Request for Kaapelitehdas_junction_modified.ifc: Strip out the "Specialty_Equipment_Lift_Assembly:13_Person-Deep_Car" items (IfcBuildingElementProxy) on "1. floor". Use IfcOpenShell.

First a look at what the model holds.

```python
import ifcopenshell
import ifcopenshell.util.element

model = ifcopenshell.open("Kaapelitehdas_junction_modified.ifc")
print(model.schema)
storey = next(s for s in model.by_type("IfcBuildingStorey") if s.Name == "1. floor")
proxies = [e for e in ifcopenshell.util.element.get_decomposition(storey) if e.is_a("IfcBuildingElementProxy")]
seen = {}
for e in proxies:
    element_type = ifcopenshell.util.element.get_type(e)
    name = element_type.Name if element_type not in (None, e) else None
    seen[name] = seen.get(name, 0) + 1
for name, count in sorted(seen.items(), key=str):
    print(count, "x", name)
```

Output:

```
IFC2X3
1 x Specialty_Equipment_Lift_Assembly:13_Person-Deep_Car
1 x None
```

```python
import ifcopenshell
import ifcopenshell.api.root
import ifcopenshell.util.element

model = ifcopenshell.open("Kaapelitehdas_junction_modified.ifc")

storey = next(s for s in model.by_type("IfcBuildingStorey") if s.Name == "1. floor")
proxies = [e for e in ifcopenshell.util.element.get_decomposition(storey) if e.is_a("IfcBuildingElementProxy")]
targets = [e for e in proxies if (t := ifcopenshell.util.element.get_type(e)) not in (None, e) and t.Name == "Specialty_Equipment_Lift_Assembly:13_Person-Deep_Car"]

for e in targets:
    ifcopenshell.api.root.remove_product(model, product=e)
print(len(targets), "removed")

model.write("Kaapelitehdas_junction_modified_rev.ifc")
```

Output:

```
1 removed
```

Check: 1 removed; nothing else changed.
